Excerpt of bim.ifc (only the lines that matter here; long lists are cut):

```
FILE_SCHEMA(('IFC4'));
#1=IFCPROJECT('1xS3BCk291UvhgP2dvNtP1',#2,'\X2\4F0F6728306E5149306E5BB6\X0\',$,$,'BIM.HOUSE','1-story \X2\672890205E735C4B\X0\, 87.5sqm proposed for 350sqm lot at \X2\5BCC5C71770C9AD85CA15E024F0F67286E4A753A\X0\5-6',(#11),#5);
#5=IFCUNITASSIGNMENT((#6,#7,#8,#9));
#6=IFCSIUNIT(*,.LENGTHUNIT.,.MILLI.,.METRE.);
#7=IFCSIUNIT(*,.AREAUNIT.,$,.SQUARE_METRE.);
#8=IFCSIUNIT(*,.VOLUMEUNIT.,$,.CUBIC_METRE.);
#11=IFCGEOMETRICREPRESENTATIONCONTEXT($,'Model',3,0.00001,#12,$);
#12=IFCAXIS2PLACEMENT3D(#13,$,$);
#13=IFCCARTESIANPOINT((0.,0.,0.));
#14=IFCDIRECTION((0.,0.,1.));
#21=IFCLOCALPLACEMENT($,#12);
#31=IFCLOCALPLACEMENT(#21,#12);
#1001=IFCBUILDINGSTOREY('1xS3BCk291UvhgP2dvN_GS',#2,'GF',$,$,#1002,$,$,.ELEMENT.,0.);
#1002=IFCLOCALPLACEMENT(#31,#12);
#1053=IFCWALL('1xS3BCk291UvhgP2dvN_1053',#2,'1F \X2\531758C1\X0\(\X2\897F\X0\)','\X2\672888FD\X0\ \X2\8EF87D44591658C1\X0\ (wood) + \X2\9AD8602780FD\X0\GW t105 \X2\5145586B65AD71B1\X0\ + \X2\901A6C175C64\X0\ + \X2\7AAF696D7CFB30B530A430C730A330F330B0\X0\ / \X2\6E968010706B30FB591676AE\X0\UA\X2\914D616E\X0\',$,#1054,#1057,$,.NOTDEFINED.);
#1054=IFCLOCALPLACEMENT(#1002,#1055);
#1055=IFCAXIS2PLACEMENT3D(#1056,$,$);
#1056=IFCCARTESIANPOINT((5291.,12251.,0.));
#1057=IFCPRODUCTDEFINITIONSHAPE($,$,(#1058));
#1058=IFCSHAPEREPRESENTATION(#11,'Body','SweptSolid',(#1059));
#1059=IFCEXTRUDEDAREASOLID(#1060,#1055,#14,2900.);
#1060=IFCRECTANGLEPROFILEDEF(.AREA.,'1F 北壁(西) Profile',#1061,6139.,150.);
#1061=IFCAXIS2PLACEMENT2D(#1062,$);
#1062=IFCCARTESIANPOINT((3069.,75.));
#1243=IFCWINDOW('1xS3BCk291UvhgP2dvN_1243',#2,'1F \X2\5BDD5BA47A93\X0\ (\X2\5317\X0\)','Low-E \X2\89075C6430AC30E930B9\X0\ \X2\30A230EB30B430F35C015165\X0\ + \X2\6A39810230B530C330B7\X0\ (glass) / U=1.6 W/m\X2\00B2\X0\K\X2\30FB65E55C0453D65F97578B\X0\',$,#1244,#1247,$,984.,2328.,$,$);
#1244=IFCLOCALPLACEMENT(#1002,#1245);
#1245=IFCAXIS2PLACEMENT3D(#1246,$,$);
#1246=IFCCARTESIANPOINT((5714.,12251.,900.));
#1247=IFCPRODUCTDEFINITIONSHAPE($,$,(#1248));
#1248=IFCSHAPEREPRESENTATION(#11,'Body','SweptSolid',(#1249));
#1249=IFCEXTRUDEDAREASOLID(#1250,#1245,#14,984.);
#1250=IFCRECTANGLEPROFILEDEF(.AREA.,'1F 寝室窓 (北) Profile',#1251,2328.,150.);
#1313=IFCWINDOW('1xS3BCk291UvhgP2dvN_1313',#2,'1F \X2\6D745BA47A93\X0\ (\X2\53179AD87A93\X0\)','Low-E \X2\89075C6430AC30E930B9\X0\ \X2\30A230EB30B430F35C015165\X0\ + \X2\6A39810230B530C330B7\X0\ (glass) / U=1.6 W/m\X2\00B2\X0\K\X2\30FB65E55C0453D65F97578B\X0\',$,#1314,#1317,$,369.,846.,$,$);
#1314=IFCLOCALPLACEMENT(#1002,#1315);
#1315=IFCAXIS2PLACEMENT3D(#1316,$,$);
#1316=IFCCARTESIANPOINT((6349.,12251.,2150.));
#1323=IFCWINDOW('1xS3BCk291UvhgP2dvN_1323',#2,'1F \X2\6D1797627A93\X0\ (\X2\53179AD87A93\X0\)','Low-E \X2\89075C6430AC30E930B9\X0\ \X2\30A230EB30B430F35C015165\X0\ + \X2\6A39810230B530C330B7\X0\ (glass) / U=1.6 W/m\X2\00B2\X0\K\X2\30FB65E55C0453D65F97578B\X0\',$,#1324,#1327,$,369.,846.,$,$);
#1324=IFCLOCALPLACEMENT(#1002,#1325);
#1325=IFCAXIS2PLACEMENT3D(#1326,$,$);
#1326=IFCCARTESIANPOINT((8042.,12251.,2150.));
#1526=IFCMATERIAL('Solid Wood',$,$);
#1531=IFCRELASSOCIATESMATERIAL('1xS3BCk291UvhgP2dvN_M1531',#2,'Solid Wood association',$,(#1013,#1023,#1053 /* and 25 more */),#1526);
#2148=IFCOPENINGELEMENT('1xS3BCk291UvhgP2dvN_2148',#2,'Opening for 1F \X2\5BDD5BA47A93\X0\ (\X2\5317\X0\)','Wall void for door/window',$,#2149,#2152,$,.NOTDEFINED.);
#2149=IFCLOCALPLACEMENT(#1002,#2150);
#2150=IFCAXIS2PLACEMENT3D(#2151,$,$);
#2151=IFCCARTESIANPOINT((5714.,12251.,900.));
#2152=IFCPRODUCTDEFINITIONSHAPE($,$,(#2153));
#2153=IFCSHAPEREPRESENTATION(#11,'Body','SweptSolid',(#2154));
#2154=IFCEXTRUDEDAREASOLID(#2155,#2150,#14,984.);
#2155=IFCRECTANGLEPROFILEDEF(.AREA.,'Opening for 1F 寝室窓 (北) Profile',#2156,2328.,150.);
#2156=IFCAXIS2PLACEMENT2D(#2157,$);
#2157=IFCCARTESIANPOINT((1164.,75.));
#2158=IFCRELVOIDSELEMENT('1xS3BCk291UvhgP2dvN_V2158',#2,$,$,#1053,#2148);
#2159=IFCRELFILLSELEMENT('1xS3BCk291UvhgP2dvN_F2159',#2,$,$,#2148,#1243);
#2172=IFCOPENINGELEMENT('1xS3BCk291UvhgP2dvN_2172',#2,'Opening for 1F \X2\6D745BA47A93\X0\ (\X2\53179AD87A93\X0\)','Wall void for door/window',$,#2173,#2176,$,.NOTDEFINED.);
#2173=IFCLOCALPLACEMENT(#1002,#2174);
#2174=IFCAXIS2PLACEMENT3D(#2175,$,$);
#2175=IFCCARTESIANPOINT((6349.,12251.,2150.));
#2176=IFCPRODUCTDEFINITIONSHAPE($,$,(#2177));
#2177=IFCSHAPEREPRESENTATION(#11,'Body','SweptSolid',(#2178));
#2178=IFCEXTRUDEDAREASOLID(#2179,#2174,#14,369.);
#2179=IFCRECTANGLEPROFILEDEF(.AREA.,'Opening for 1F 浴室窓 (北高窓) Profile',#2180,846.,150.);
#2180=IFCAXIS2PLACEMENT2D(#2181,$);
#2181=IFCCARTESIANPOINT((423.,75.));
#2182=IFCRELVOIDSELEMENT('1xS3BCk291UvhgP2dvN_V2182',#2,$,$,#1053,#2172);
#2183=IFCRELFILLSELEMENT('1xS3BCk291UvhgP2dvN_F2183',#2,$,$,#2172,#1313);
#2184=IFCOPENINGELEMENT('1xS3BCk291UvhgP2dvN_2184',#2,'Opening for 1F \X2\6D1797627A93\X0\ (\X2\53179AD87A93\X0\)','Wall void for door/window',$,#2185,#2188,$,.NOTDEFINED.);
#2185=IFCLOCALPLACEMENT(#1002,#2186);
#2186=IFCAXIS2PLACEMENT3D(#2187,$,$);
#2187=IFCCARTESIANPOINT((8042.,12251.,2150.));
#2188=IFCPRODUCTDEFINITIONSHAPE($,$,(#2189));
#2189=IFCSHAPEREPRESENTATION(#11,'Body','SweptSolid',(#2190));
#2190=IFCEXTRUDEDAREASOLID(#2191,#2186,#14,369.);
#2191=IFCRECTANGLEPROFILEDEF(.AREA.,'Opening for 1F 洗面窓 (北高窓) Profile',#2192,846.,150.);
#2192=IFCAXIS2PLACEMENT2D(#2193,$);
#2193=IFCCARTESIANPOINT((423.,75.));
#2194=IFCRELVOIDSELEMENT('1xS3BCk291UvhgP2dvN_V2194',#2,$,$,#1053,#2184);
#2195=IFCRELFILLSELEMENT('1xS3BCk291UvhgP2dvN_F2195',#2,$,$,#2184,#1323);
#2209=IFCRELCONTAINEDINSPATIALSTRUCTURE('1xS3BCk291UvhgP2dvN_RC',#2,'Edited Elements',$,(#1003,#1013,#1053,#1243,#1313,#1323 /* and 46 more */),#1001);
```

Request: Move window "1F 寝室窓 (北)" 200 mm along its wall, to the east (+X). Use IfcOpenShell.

```python
import ifcopenshell
import ifcopenshell.api.geometry
import ifcopenshell.util.placement

model = ifcopenshell.open("bim.ifc")

window = model.by_guid("1xS3BCk291UvhgP2dvN_1243")
opening = window.FillsVoids[0].RelatingOpeningElement
wall = opening.VoidsElements[0].RelatingBuildingElement

wall_matrix = ifcopenshell.util.placement.get_local_placement(wall.ObjectPlacement)
shift = wall_matrix[:3, 0] * 200.0
before = ifcopenshell.util.placement.get_local_placement(window.ObjectPlacement)[:3, 3].copy()

# The window is not placed relative to its opening, so move both.
for product in (opening, window):
    matrix = ifcopenshell.util.placement.get_local_placement(product.ObjectPlacement)
    matrix[:3, 3] += shift
    ifcopenshell.api.geometry.edit_object_placement(model, product=product, matrix=matrix, is_si=False)

after = ifcopenshell.util.placement.get_local_placement(window.ObjectPlacement)[:3, 3]
print("window moved by", (after - before).round(3) + 0.0)

model.write("bim_updated.ifc")
```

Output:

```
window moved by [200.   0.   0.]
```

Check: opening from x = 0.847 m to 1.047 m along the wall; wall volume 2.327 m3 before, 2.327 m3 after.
